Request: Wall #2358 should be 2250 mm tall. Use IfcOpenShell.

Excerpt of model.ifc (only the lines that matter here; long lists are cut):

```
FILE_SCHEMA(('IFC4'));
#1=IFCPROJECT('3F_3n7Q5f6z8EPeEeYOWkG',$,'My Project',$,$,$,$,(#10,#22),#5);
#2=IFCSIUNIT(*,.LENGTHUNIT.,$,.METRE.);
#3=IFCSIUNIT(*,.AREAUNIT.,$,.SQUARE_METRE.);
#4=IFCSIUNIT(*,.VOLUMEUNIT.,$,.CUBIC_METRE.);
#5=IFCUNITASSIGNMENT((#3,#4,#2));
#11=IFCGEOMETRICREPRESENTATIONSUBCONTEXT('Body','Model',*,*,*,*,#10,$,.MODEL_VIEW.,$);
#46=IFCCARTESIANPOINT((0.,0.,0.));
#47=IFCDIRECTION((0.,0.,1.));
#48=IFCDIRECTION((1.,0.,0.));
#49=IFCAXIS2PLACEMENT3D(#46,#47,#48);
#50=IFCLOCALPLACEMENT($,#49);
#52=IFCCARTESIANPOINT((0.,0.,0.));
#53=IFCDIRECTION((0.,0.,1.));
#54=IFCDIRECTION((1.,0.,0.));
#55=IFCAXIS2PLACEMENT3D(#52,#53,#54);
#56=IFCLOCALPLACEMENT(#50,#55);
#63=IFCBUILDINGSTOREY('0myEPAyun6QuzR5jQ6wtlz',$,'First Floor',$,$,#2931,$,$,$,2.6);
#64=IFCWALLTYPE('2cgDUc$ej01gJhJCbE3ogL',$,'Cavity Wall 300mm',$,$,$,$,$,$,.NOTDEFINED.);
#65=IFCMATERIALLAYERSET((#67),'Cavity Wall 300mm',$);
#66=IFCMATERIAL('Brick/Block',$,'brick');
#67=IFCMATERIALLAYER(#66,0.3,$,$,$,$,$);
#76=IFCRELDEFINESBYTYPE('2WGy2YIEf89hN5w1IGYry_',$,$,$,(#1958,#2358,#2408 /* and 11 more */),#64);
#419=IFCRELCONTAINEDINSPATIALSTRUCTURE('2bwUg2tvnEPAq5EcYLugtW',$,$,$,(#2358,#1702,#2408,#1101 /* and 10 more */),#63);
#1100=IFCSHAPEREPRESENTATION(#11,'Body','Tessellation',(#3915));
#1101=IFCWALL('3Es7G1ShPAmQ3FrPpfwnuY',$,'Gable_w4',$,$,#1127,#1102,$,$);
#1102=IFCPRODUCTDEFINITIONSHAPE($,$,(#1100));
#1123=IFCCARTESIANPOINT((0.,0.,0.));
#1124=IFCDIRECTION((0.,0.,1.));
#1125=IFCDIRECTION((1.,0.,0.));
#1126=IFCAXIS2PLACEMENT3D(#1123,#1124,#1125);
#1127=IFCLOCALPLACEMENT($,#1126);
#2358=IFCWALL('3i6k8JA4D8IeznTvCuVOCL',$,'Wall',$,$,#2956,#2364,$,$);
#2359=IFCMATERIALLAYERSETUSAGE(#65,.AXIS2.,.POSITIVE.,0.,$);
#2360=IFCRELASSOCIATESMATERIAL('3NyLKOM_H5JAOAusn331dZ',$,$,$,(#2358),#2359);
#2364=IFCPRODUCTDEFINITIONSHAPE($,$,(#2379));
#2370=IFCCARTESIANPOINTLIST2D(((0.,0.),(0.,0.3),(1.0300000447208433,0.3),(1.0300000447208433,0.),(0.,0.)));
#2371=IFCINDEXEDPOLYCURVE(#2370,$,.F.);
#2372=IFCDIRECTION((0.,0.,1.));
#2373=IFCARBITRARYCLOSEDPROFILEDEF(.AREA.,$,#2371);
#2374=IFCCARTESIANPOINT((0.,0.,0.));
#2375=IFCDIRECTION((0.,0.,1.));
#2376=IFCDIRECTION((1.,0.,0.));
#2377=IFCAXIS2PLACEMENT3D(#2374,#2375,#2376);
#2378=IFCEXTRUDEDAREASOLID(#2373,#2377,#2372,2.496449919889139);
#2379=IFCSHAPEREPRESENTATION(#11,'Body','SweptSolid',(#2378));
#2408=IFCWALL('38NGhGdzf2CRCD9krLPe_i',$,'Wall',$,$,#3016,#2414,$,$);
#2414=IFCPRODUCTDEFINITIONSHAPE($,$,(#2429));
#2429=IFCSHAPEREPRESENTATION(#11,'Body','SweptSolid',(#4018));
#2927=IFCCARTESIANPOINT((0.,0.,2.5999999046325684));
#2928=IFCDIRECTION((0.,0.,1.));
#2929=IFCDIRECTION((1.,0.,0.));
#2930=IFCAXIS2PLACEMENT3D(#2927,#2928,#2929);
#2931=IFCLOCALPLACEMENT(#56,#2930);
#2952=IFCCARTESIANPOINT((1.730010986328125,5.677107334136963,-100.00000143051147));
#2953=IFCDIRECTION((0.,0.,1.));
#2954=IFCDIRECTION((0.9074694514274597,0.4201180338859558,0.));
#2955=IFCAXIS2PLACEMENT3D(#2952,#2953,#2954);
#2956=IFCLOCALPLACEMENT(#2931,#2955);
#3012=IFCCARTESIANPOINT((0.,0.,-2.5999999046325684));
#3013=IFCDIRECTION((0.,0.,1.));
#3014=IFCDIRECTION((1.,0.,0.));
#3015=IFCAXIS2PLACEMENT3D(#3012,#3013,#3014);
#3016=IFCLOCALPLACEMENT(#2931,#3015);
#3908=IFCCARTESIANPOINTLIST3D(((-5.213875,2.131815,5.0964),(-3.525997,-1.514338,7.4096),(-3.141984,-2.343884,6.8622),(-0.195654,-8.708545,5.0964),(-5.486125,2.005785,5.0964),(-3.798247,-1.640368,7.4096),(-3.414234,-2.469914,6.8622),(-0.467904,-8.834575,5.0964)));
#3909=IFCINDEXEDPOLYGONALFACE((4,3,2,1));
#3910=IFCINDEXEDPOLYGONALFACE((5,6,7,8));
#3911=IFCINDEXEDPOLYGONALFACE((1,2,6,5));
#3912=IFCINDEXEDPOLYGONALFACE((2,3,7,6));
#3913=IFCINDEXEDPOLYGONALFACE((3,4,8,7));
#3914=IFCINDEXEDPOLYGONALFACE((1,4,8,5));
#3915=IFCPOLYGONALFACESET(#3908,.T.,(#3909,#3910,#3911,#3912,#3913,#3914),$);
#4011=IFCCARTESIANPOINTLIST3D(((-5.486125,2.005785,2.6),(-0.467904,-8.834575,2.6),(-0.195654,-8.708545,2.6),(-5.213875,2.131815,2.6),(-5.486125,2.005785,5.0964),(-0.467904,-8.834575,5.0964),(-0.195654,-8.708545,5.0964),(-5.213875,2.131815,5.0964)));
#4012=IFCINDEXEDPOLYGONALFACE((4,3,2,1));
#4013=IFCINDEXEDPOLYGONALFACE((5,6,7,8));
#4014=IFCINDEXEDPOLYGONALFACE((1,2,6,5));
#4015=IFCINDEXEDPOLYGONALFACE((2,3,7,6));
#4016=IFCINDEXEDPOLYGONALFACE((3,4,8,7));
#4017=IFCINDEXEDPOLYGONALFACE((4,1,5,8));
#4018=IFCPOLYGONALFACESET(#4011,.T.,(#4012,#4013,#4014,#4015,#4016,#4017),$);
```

```python
import ifcopenshell
import ifcopenshell.geom
import ifcopenshell.util.representation
import ifcopenshell.util.shape

model = ifcopenshell.open("model.ifc")
settings = ifcopenshell.geom.settings()


def volume(element):
    """Net volume in cubic metres, openings subtracted."""
    shape = ifcopenshell.geom.create_shape(settings, element)
    return ifcopenshell.util.shape.get_volume(shape.geometry)


wall = model.by_guid("3i6k8JA4D8IeznTvCuVOCL")
before = volume(wall)

body = ifcopenshell.util.representation.get_representation(wall, "Model", "Body")
solid = body.Items[0]
old_height = solid.Depth
solid.Depth = 2.25
after = volume(wall)

print(f"height {old_height:g} -> {solid.Depth:g}, volume {before:.3f} -> {after:.3f} m3")

model.write("model_rev.ifc")
```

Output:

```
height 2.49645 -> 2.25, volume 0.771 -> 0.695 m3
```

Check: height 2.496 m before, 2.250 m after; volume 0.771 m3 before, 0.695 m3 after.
